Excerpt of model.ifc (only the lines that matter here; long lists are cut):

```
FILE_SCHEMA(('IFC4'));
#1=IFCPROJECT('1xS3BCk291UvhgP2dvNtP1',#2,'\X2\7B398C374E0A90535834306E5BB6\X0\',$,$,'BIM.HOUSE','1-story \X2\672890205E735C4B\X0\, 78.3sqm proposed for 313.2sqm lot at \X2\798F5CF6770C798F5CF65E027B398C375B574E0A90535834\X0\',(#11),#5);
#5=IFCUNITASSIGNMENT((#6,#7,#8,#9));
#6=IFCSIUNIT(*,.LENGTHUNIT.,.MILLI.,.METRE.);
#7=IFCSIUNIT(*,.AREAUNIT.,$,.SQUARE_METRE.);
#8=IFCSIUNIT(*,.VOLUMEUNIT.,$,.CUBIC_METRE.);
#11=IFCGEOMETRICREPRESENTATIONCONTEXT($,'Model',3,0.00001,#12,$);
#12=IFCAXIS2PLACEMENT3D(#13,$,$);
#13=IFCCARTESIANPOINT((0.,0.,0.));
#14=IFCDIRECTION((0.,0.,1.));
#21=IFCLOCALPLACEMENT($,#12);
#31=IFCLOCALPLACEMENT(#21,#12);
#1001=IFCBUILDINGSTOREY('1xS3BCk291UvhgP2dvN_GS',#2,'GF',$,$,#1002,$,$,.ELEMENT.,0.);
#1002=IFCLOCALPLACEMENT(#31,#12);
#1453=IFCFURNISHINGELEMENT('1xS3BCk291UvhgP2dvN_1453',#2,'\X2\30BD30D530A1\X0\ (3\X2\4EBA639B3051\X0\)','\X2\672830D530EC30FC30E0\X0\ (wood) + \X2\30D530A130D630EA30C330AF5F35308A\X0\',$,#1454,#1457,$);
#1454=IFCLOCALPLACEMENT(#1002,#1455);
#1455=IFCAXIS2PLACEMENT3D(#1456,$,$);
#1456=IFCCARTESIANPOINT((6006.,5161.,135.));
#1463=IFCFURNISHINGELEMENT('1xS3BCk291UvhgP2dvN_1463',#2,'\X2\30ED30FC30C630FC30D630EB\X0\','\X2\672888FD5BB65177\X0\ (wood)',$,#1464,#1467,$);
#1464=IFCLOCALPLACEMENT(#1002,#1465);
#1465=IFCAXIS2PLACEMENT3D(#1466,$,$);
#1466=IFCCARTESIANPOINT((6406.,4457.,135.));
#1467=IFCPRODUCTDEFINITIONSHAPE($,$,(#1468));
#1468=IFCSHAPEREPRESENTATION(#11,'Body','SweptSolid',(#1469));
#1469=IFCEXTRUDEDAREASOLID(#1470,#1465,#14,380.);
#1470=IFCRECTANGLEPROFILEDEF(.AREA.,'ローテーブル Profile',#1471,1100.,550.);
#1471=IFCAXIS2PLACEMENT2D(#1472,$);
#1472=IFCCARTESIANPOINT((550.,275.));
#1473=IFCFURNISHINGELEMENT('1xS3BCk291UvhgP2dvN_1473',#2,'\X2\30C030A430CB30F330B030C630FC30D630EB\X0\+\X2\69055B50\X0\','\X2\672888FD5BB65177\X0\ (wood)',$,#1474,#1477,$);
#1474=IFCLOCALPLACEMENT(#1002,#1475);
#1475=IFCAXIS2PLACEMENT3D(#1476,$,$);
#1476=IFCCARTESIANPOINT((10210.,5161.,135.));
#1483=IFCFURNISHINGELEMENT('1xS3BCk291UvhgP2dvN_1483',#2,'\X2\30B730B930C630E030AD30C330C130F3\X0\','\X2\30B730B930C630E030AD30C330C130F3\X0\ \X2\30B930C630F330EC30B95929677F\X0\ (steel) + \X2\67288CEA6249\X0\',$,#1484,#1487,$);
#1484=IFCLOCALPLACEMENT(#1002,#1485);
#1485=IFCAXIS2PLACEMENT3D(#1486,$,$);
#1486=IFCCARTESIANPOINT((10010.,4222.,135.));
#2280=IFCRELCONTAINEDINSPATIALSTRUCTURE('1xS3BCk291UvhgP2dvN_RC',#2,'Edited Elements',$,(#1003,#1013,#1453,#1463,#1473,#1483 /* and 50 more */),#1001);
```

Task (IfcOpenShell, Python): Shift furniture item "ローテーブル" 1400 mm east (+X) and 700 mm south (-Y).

```python
import ifcopenshell
import ifcopenshell.api.geometry
import ifcopenshell.util.placement
import ifcopenshell.util.unit

model = ifcopenshell.open("model.ifc")
unit_scale = ifcopenshell.util.unit.calculate_unit_scale(model)

item = model.by_guid("1xS3BCk291UvhgP2dvN_1463")
matrix = ifcopenshell.util.placement.get_local_placement(item.ObjectPlacement)
matrix[0, 3] += 1.4 / unit_scale
matrix[1, 3] -= 0.7 / unit_scale
ifcopenshell.api.geometry.edit_object_placement(model, product=item, matrix=matrix, is_si=False)

print(ifcopenshell.util.placement.get_local_placement(item.ObjectPlacement).round(3) + 0.0)

model.write("model_edited.ifc")
```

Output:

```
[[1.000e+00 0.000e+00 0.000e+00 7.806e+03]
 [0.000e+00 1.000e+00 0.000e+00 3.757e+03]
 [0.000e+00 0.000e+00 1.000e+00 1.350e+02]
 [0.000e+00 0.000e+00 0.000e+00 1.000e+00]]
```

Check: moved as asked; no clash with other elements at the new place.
